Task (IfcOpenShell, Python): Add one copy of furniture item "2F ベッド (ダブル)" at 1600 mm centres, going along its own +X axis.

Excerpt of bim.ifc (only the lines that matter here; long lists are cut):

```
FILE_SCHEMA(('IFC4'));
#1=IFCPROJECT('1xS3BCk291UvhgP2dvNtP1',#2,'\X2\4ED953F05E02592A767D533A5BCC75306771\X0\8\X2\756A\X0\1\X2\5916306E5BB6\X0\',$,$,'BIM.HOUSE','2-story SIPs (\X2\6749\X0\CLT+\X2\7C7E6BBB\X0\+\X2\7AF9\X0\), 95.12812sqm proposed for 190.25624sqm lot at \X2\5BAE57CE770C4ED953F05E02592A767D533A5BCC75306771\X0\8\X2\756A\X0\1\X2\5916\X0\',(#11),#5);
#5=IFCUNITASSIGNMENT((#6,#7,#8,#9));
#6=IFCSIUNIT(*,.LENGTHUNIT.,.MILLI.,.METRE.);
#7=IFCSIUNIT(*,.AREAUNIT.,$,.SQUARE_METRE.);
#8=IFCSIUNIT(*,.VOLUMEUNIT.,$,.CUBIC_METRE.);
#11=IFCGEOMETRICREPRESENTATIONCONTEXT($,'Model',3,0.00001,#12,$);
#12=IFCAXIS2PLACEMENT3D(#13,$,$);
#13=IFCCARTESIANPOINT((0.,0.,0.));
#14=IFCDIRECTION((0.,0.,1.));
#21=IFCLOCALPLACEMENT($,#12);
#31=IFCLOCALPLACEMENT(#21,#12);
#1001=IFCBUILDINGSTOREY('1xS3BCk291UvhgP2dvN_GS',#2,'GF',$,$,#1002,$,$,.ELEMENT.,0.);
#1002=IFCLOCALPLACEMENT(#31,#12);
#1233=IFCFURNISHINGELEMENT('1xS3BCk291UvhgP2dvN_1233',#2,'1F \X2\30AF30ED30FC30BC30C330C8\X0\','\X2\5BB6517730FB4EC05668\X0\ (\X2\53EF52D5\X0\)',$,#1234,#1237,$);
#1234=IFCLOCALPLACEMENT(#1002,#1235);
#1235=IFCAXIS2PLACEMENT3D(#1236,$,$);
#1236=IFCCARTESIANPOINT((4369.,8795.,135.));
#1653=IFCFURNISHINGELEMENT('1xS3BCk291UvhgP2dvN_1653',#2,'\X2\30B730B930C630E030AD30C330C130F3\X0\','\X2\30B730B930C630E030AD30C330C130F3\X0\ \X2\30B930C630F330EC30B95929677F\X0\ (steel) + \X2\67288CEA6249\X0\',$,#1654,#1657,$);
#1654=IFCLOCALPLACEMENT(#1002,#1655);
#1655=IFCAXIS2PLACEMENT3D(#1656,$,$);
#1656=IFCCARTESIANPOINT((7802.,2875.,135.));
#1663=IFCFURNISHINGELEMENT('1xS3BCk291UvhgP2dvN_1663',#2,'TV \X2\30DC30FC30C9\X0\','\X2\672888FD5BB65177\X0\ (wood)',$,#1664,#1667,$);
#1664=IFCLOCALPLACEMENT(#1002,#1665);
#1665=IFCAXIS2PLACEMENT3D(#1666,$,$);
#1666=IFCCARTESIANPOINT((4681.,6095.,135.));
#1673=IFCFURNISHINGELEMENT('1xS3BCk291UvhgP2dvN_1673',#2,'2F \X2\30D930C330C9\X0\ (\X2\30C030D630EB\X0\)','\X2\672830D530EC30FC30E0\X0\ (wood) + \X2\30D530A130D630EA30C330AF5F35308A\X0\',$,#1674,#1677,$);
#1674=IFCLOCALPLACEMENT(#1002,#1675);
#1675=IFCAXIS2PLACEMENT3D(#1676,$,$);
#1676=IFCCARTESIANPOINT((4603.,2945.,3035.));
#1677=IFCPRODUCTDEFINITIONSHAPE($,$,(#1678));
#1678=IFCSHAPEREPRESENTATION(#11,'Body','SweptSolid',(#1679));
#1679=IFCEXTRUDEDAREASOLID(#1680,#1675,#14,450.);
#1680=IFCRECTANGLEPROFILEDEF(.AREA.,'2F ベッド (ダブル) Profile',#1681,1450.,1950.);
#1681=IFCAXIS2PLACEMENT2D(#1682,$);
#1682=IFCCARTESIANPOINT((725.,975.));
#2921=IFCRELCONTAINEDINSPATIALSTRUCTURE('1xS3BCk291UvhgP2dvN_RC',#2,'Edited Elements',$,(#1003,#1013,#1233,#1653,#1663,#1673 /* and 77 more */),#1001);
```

```python
import ifcopenshell
import ifcopenshell.api.geometry
import ifcopenshell.api.root
import ifcopenshell.util.element
import ifcopenshell.util.placement
import ifcopenshell.util.unit

model = ifcopenshell.open("bim.ifc")
unit_scale = ifcopenshell.util.unit.calculate_unit_scale(model)


def reuse_history(source, copy):
    """copy_class also copies each property set's owner history, people and application; keep the originals."""
    for rel in copy.IsDefinedBy:
        if rel.is_a("IfcRelDefinesByProperties") and (history := rel.RelatingPropertyDefinition.OwnerHistory):
            rel.RelatingPropertyDefinition.OwnerHistory = source.OwnerHistory
            ifcopenshell.util.element.remove_deep2(model, history)


source = model.by_guid("1xS3BCk291UvhgP2dvN_1673")
base = ifcopenshell.util.placement.get_local_placement(source.ObjectPlacement)
step = base[:3, 0] * 1.6 / unit_scale

for i in range(1, 2):
    copy = ifcopenshell.api.root.copy_class(model, product=source)
    copy.Representation = ifcopenshell.util.element.copy_deep(
        model, source.Representation, exclude=["IfcGeometricRepresentationContext", "IfcRepresentationMap"]
    )
    reuse_history(source, copy)
    matrix = base.copy()
    matrix[:3, 3] += i * step
    print("added at", matrix[:3, 3].round(3) + 0.0)
    ifcopenshell.api.geometry.edit_object_placement(model, product=copy, matrix=matrix, is_si=False)

model.write("bim-out.ifc")
```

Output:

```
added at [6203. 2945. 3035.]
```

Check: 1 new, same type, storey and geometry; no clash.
